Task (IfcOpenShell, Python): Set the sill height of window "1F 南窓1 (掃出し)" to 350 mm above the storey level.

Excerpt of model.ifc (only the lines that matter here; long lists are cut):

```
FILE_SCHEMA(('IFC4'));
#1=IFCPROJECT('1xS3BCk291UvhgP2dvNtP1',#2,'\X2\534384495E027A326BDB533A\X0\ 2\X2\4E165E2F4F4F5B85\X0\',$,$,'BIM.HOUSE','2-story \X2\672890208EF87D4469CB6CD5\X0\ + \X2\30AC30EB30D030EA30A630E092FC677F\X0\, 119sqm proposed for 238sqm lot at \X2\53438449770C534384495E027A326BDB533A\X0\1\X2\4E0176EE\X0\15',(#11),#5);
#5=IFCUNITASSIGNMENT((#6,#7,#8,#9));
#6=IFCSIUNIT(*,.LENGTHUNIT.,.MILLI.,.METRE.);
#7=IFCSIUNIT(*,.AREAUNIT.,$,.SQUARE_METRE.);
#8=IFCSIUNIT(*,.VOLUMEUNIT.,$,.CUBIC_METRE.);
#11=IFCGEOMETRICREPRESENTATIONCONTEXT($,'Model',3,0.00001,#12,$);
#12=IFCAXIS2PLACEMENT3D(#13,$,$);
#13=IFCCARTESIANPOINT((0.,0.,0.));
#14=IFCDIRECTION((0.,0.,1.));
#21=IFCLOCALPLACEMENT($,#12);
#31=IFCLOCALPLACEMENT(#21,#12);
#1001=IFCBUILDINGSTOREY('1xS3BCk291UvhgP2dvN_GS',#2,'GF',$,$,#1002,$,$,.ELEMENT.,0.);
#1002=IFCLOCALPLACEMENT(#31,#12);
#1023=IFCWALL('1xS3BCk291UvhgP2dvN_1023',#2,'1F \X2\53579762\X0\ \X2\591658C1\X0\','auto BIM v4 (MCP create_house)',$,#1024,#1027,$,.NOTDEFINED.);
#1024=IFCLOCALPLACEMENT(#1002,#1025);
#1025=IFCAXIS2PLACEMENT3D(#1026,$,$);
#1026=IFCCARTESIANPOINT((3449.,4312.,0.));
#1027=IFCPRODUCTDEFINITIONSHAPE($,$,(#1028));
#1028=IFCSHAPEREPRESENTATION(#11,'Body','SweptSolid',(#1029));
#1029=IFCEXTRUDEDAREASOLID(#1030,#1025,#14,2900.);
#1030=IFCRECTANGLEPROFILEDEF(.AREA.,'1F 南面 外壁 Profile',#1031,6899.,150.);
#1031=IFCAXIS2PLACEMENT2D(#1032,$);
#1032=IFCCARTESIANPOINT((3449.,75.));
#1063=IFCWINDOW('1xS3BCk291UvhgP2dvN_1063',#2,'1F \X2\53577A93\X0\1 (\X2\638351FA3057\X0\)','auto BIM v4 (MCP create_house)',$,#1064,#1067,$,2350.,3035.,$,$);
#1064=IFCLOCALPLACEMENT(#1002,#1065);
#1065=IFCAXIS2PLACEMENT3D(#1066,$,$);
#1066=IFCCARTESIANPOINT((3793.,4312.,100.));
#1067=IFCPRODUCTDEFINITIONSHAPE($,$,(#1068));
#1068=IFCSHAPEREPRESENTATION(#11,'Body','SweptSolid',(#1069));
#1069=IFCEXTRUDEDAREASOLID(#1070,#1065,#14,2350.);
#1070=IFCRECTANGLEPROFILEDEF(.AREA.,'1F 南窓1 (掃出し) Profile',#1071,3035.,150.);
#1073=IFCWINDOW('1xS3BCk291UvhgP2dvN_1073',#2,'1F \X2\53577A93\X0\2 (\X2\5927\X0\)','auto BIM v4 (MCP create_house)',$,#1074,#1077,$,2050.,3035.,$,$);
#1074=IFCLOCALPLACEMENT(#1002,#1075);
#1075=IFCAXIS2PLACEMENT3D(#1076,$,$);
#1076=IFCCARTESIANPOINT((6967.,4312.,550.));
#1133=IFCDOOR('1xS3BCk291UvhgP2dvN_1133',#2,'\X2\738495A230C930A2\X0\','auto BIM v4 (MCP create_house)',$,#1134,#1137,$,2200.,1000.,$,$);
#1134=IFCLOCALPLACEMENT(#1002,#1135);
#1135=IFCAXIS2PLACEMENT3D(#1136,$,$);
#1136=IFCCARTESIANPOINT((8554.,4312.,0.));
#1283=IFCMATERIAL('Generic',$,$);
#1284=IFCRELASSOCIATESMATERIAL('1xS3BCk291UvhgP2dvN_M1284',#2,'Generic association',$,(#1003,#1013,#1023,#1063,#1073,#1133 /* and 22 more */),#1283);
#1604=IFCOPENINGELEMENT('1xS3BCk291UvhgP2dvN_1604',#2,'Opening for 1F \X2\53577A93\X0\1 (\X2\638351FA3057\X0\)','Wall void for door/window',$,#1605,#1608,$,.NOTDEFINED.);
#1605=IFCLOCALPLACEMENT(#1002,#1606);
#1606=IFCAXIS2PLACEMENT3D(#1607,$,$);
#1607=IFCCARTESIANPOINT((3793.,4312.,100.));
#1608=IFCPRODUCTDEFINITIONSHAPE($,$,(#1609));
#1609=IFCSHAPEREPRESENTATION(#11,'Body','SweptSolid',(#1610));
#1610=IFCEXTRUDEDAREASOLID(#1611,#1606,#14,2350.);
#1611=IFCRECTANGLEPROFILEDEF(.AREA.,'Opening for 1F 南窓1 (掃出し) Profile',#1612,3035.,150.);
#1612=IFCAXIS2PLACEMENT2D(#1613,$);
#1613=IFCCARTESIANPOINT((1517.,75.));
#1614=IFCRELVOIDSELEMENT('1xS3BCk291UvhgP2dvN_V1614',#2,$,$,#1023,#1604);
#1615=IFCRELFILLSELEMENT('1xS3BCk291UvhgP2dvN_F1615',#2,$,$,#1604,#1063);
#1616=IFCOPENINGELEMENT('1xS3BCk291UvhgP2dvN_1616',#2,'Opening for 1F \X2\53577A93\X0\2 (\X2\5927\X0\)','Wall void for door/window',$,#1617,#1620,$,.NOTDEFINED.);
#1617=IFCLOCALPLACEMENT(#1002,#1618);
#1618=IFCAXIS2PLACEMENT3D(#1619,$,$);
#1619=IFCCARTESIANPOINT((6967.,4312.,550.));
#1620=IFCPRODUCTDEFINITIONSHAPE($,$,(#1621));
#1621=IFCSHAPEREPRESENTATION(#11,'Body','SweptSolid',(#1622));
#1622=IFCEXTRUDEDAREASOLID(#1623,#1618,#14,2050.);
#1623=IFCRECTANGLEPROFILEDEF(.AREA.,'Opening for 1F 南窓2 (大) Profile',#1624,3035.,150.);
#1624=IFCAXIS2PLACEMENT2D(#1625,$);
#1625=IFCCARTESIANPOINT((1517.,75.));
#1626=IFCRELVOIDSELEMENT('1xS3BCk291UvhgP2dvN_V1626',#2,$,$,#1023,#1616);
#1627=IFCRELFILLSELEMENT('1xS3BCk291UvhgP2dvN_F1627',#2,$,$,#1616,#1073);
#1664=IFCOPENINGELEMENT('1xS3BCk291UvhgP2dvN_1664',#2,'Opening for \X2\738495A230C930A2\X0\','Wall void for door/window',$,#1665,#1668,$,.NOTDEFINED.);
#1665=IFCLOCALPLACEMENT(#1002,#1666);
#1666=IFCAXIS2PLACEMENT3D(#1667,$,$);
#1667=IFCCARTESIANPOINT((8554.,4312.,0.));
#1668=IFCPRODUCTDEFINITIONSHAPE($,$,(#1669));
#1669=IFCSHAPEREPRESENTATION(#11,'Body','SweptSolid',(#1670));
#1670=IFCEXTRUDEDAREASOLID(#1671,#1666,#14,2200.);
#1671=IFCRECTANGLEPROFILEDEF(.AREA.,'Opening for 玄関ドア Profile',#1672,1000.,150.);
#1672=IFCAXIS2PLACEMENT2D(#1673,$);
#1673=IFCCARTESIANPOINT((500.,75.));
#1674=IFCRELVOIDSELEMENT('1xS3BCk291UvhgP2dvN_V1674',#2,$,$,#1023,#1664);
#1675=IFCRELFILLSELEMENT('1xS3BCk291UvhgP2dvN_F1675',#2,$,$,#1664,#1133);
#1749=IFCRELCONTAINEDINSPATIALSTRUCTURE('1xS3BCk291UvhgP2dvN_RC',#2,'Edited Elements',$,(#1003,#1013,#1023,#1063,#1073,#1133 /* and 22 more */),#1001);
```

```python
import numpy as np
import ifcopenshell
import ifcopenshell.api.geometry
import ifcopenshell.geom
import ifcopenshell.util.element
import ifcopenshell.util.placement
import ifcopenshell.util.shape
import ifcopenshell.util.unit

model = ifcopenshell.open("model.ifc")
unit_scale = ifcopenshell.util.unit.calculate_unit_scale(model)

window = model.by_id(1063)
opening = window.FillsVoids[0].RelatingOpeningElement
storey = ifcopenshell.util.element.get_container(window, ifc_class="IfcBuildingStorey")
level = ifcopenshell.util.placement.get_local_placement(storey.ObjectPlacement)[2, 3]

# The opening's origin need not be at the sill, so measure its lowest point.
shape = ifcopenshell.geom.create_shape(ifcopenshell.geom.settings(), opening)
bottom = ifcopenshell.util.shape.get_shape_bottom_elevation(shape, shape.geometry) / unit_scale
dz = level + 350.0 - bottom

shift = np.array([0.0, 0.0, dz])
# The window is not placed relative to its opening, so move both.
for product in (opening, window):
    matrix = ifcopenshell.util.placement.get_local_placement(product.ObjectPlacement)
    matrix[:3, 3] += shift
    ifcopenshell.api.geometry.edit_object_placement(model, product=product, matrix=matrix, is_si=False)

print(f"moved by {dz * unit_scale:+.3f} m")

model.write("model_edited.ifc")
```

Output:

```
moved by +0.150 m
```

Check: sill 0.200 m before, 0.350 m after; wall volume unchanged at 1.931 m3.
